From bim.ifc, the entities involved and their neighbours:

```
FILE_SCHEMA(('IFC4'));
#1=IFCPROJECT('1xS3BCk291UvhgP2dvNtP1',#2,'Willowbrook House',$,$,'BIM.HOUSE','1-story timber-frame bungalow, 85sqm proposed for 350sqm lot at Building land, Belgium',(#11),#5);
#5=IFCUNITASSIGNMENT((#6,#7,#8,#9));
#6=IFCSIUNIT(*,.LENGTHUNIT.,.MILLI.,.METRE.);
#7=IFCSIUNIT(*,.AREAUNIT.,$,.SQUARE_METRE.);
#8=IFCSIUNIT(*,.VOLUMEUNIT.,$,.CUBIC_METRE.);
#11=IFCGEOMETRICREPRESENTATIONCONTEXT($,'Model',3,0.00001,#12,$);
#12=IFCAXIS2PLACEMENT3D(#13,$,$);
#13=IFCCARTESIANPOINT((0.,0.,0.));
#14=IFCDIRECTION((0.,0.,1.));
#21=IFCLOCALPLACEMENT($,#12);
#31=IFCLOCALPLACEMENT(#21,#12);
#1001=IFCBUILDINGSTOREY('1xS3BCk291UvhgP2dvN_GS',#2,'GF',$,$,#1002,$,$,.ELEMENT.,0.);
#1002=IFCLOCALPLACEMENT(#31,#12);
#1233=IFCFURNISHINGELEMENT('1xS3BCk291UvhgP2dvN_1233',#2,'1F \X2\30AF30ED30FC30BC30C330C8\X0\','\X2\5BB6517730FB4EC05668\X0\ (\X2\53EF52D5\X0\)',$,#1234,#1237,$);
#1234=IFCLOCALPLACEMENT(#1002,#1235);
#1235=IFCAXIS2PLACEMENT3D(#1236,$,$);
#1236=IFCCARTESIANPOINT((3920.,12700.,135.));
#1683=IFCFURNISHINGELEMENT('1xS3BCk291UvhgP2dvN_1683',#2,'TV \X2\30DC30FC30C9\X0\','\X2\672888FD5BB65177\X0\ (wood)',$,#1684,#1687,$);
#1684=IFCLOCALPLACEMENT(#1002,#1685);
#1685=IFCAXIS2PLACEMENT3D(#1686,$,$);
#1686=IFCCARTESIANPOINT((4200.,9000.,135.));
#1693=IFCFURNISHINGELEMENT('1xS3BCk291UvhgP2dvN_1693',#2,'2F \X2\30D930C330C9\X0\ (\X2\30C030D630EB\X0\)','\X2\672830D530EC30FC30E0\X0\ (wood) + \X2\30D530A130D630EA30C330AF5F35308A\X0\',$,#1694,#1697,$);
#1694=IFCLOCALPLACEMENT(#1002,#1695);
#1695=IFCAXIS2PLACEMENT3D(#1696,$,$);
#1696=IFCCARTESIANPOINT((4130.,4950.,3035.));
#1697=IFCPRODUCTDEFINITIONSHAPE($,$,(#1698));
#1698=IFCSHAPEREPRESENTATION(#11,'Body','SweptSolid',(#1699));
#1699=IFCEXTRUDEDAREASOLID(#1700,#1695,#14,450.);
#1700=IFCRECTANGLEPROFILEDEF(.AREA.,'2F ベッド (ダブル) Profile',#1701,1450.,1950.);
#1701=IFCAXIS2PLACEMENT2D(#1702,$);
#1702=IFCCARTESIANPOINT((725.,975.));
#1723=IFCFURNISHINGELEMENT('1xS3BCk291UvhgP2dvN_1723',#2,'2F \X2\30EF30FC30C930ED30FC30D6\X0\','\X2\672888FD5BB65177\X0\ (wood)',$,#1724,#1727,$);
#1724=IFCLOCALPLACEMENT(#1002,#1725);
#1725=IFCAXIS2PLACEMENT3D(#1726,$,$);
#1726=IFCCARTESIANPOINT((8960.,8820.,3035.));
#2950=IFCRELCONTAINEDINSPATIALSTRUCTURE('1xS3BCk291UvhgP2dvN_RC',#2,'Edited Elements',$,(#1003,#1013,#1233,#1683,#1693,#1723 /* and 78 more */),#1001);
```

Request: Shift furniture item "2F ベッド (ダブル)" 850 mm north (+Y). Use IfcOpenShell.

```python
import ifcopenshell
import ifcopenshell.api.geometry
import ifcopenshell.util.placement
import ifcopenshell.util.unit

model = ifcopenshell.open("bim.ifc")
unit_scale = ifcopenshell.util.unit.calculate_unit_scale(model)

item = model.by_guid("1xS3BCk291UvhgP2dvN_1693")
matrix = ifcopenshell.util.placement.get_local_placement(item.ObjectPlacement)
matrix[1, 3] += 0.85 / unit_scale
ifcopenshell.api.geometry.edit_object_placement(model, product=item, matrix=matrix, is_si=False)

print(ifcopenshell.util.placement.get_local_placement(item.ObjectPlacement).round(3) + 0.0)

model.write("bim_rev.ifc")
```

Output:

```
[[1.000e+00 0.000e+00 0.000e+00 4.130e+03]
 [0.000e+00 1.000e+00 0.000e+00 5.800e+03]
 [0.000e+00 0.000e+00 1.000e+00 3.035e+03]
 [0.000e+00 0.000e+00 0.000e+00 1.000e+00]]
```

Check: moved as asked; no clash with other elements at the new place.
